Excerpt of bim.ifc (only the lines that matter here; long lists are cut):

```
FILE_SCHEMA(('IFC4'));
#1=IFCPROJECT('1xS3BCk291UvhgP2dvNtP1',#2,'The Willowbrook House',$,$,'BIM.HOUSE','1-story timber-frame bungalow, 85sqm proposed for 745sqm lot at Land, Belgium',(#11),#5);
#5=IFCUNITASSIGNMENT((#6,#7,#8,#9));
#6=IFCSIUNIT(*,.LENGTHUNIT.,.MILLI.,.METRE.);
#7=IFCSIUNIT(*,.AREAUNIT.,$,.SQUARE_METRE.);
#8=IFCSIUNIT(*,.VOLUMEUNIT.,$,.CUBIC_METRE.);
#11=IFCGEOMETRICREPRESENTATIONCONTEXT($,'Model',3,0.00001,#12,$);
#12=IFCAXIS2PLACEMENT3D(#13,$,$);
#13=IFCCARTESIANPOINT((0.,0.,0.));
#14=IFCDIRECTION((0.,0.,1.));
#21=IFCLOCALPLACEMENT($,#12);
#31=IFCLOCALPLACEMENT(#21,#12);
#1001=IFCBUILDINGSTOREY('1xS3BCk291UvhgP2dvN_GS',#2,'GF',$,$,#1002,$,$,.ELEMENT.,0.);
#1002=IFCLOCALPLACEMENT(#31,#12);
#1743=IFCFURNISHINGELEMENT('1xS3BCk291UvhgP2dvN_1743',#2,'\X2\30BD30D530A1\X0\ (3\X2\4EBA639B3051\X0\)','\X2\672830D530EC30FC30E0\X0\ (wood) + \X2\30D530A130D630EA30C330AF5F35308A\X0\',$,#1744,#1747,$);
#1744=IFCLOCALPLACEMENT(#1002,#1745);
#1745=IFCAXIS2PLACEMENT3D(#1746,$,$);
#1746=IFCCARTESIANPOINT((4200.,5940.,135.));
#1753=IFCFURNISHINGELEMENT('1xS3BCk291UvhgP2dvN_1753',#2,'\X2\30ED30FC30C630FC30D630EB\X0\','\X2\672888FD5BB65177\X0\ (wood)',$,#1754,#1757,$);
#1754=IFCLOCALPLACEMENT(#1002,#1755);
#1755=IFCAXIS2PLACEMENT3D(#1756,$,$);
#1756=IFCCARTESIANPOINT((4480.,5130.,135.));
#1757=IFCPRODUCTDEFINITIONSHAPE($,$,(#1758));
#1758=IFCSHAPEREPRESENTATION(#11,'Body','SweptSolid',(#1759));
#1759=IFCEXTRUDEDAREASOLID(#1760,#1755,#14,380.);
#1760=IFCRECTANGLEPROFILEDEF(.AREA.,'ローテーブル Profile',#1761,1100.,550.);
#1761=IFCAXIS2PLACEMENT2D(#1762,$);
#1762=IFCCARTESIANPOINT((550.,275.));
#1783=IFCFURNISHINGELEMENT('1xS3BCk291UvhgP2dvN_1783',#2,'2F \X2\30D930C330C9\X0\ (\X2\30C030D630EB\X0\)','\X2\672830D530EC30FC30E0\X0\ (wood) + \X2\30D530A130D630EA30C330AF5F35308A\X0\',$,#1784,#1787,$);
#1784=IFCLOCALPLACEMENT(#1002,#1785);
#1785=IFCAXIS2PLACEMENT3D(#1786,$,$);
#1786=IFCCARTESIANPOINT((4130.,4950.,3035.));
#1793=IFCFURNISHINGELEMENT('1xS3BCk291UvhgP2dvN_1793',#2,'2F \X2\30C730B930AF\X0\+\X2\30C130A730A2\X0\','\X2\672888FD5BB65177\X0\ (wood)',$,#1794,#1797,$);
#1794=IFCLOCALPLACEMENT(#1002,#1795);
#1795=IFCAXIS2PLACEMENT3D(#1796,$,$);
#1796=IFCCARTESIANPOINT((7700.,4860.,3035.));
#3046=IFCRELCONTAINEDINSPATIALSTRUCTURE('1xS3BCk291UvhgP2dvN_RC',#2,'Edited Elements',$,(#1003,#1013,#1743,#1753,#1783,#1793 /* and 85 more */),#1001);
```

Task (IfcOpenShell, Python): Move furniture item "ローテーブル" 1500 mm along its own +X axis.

```python
import ifcopenshell
import ifcopenshell.api.geometry
import ifcopenshell.util.placement
import ifcopenshell.util.unit

model = ifcopenshell.open("bim.ifc")
unit_scale = ifcopenshell.util.unit.calculate_unit_scale(model)

item = model.by_guid("1xS3BCk291UvhgP2dvN_1753")
matrix = ifcopenshell.util.placement.get_local_placement(item.ObjectPlacement)
matrix[:3, 3] += matrix[:3, 0] * 1.5 / unit_scale
ifcopenshell.api.geometry.edit_object_placement(model, product=item, matrix=matrix, is_si=False)

print(ifcopenshell.util.placement.get_local_placement(item.ObjectPlacement).round(3) + 0.0)

model.write("bim-out.ifc")
```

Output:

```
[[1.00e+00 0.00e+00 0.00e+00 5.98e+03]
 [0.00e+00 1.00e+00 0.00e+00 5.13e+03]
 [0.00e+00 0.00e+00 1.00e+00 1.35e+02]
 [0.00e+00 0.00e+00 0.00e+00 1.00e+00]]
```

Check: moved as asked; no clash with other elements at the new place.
